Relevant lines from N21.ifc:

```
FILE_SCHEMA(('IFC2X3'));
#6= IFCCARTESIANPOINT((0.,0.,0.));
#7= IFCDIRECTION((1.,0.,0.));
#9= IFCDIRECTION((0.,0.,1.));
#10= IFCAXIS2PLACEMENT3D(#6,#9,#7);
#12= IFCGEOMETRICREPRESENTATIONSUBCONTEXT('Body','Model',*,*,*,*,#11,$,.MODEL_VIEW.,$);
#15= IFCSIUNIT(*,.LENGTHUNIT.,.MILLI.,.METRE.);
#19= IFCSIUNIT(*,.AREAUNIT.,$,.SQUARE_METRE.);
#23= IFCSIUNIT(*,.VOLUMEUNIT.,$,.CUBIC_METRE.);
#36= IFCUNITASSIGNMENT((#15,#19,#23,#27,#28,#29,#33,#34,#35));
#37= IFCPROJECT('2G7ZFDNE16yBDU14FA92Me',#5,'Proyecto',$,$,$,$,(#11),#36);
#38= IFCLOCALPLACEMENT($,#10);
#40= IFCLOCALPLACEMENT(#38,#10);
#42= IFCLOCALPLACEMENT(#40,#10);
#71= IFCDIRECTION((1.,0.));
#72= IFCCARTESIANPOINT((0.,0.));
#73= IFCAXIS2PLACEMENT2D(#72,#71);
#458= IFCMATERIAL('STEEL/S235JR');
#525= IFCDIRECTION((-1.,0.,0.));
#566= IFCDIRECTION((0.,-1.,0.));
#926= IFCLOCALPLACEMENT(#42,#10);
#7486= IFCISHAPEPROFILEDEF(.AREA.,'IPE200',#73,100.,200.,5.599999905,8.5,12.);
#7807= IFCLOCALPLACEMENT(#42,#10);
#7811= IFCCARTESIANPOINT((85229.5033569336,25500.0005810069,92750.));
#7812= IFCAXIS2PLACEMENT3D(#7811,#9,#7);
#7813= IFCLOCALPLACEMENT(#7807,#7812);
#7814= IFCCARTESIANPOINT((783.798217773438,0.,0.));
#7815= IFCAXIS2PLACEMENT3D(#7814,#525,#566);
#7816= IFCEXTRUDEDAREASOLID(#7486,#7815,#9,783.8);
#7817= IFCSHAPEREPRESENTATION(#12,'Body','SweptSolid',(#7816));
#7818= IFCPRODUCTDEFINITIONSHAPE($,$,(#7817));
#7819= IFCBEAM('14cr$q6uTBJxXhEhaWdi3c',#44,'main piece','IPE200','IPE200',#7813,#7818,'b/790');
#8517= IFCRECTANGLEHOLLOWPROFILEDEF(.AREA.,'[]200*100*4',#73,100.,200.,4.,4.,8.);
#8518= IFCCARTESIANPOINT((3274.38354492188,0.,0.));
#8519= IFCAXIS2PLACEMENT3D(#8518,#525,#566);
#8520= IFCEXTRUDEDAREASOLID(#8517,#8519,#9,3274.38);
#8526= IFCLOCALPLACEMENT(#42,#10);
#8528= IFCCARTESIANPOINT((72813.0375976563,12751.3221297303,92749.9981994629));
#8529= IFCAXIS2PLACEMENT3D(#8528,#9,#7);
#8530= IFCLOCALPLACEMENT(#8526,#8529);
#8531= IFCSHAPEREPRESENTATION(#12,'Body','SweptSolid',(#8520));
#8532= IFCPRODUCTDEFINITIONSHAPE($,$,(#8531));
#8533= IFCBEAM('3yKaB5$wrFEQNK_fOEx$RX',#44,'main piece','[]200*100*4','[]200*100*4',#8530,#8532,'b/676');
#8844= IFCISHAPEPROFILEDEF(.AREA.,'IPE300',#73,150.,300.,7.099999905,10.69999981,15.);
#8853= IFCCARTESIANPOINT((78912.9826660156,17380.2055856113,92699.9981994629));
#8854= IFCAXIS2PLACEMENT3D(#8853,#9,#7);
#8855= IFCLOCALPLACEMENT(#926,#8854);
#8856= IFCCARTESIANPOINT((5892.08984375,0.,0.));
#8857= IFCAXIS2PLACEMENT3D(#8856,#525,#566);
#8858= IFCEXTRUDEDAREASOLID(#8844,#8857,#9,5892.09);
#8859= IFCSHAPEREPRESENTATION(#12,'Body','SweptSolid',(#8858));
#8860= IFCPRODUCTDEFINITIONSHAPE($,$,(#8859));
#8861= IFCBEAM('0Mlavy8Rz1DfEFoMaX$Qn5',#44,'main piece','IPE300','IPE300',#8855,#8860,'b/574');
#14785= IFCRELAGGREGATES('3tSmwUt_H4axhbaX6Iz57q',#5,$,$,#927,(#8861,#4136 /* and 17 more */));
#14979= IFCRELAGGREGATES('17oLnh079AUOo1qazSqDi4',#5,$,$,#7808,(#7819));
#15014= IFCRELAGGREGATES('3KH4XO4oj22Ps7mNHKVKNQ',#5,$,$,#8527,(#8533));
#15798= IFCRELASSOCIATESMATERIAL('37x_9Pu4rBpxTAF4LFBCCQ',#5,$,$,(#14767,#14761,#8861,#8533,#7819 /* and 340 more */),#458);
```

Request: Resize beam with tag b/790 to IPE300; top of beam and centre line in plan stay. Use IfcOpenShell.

```python
import ifcopenshell
import ifcopenshell.util.element
import ifcopenshell.util.representation

model = ifcopenshell.open("N21.ifc")

member = model.by_guid("14cr$q6uTBJxXhEhaWdi3c")
source = next(p for p in model.by_type("IfcIShapeProfileDef") if p.ProfileName == "IPE300")

body = ifcopenshell.util.representation.get_representation(member, "Model", "Body")
solid = body.Items[0]
old_profile = solid.SweptArea

# Copy the section's sizes but keep this member's own profile position.
profile = ifcopenshell.util.element.copy(model, source)
# Profiles are centred, so shift by half the change in depth to hold the top.
shift = (old_profile.OverallDepth - profile.OverallDepth) / 2
x, y = old_profile.Position.Location.Coordinates
up = (0.0, 1.0)  # upwards, in the solid's own plane
location = model.createIfcCartesianPoint((x + up[0] * shift, y + up[1] * shift))
profile.Position = model.createIfcAxis2Placement2D(location, old_profile.Position.RefDirection)
solid.SweptArea = profile
if not model.get_total_inverses(old_profile):
    ifcopenshell.util.element.remove_deep2(model, old_profile)
member.Description = member.Description.replace("IPE200", "IPE300")
member.ObjectType = member.ObjectType.replace("IPE200", "IPE300")

print(solid.SweptArea)

model.write("N21_updated.ifc")
```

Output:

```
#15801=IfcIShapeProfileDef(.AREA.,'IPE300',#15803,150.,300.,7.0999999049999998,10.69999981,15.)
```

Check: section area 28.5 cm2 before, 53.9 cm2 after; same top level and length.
